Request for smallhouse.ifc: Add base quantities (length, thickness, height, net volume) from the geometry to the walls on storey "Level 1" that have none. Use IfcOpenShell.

First a look at what the model holds.

```python
import ifcopenshell
import ifcopenshell.util.element
import ifcopenshell.util.unit

model = ifcopenshell.open("smallhouse.ifc")
print(model.schema)
for unit_type in ("LENGTHUNIT", "AREAUNIT", "VOLUMEUNIT"):
    print(unit_type, ifcopenshell.util.unit.calculate_unit_scale(model, unit_type))
storey = next(s for s in model.by_type("IfcBuildingStorey") if s.Name == "Level 1")
walls = [e for e in ifcopenshell.util.element.get_decomposition(storey) if e.is_a("IfcWall")]
for e in sorted(walls, key=lambda e: e.id()):
    print(e.id(), e.is_a(), e.Name, list(ifcopenshell.util.element.get_psets(e, qtos_only=True)), sep=" | ")
```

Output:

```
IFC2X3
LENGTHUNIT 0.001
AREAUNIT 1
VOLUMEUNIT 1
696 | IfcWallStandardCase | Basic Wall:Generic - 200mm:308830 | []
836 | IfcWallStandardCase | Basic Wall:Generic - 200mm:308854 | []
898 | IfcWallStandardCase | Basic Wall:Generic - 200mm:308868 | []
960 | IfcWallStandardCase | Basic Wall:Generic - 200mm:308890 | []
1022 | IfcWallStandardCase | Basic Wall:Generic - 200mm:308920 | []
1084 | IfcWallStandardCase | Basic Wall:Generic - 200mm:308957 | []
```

```python
import ifcopenshell
import ifcopenshell.api.pset
import ifcopenshell.geom
import ifcopenshell.util.element
import ifcopenshell.util.shape
import ifcopenshell.util.unit

model = ifcopenshell.open("smallhouse.ifc")
unit_scale = ifcopenshell.util.unit.calculate_unit_scale(model)
volume_scale = ifcopenshell.util.unit.calculate_unit_scale(model, "VOLUMEUNIT")
settings = ifcopenshell.geom.settings()

storey = next(s for s in model.by_type("IfcBuildingStorey") if s.Name == "Level 1")
walls = [e for e in ifcopenshell.util.element.get_decomposition(storey) if e.is_a("IfcWall")]

for e in sorted(walls, key=lambda e: e.id()):
    if ifcopenshell.util.element.get_psets(e, qtos_only=True, should_inherit=False):
        continue
    # Geometry comes back in metres, in the element's own axes.
    shape = ifcopenshell.geom.create_shape(settings, e)
    values = {
        "Length": ifcopenshell.util.shape.get_x(shape.geometry) / unit_scale,
        "Width": ifcopenshell.util.shape.get_y(shape.geometry) / unit_scale,
        "Height": ifcopenshell.util.shape.get_z(shape.geometry) / unit_scale,
        "NetVolume": ifcopenshell.util.shape.get_volume(shape.geometry) / volume_scale,
    }
    qto = ifcopenshell.api.pset.add_qto(model, product=e, name="BaseQuantities")
    ifcopenshell.api.pset.edit_qto(model, qto=qto, properties=values)
    print(e.id(), {k: round(v, 3) for k, v in values.items()})

model.write("smallhouse_updated.ifc")
```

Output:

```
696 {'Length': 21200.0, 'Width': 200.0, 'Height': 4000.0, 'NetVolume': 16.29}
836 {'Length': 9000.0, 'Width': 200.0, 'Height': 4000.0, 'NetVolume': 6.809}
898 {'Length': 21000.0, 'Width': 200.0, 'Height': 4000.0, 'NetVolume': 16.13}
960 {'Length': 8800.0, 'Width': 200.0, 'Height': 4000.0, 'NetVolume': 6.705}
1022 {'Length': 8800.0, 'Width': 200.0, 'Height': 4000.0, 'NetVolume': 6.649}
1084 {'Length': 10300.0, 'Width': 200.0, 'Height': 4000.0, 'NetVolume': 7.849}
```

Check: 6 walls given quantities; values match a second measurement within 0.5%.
